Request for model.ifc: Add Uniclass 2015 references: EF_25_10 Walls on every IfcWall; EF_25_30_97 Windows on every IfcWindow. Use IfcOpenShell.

First a look at what the model holds.

```python
import ifcopenshell

model = ifcopenshell.open("model.ifc")
print(model.schema)
print("classifications:", [c.Name for c in model.by_type("IfcClassification")])
for ifc_class in ("IfcDoor", "IfcRoof", "IfcStair", "IfcWall", "IfcWindow"):
    print(ifc_class, len(model.by_type(ifc_class)))
```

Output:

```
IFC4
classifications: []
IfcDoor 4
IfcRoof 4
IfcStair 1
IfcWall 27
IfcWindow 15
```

```python
import ifcopenshell
import ifcopenshell.api.classification

model = ifcopenshell.open("model.ifc")

system = ifcopenshell.api.classification.add_classification(model, classification="Uniclass 2015")

codes = {
    "IfcWall": ("EF_25_10", "Walls"),
    "IfcWindow": ("EF_25_30_97", "Windows"),
}
for ifc_class, (code, name) in codes.items():
    products = model.by_type(ifc_class)
    ifcopenshell.api.classification.add_reference(
        model, products=products, classification=system, identification=code, name=name
    )
    print(code, len(products))

model.write("model_updated.ifc")
```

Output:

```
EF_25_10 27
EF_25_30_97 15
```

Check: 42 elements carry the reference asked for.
